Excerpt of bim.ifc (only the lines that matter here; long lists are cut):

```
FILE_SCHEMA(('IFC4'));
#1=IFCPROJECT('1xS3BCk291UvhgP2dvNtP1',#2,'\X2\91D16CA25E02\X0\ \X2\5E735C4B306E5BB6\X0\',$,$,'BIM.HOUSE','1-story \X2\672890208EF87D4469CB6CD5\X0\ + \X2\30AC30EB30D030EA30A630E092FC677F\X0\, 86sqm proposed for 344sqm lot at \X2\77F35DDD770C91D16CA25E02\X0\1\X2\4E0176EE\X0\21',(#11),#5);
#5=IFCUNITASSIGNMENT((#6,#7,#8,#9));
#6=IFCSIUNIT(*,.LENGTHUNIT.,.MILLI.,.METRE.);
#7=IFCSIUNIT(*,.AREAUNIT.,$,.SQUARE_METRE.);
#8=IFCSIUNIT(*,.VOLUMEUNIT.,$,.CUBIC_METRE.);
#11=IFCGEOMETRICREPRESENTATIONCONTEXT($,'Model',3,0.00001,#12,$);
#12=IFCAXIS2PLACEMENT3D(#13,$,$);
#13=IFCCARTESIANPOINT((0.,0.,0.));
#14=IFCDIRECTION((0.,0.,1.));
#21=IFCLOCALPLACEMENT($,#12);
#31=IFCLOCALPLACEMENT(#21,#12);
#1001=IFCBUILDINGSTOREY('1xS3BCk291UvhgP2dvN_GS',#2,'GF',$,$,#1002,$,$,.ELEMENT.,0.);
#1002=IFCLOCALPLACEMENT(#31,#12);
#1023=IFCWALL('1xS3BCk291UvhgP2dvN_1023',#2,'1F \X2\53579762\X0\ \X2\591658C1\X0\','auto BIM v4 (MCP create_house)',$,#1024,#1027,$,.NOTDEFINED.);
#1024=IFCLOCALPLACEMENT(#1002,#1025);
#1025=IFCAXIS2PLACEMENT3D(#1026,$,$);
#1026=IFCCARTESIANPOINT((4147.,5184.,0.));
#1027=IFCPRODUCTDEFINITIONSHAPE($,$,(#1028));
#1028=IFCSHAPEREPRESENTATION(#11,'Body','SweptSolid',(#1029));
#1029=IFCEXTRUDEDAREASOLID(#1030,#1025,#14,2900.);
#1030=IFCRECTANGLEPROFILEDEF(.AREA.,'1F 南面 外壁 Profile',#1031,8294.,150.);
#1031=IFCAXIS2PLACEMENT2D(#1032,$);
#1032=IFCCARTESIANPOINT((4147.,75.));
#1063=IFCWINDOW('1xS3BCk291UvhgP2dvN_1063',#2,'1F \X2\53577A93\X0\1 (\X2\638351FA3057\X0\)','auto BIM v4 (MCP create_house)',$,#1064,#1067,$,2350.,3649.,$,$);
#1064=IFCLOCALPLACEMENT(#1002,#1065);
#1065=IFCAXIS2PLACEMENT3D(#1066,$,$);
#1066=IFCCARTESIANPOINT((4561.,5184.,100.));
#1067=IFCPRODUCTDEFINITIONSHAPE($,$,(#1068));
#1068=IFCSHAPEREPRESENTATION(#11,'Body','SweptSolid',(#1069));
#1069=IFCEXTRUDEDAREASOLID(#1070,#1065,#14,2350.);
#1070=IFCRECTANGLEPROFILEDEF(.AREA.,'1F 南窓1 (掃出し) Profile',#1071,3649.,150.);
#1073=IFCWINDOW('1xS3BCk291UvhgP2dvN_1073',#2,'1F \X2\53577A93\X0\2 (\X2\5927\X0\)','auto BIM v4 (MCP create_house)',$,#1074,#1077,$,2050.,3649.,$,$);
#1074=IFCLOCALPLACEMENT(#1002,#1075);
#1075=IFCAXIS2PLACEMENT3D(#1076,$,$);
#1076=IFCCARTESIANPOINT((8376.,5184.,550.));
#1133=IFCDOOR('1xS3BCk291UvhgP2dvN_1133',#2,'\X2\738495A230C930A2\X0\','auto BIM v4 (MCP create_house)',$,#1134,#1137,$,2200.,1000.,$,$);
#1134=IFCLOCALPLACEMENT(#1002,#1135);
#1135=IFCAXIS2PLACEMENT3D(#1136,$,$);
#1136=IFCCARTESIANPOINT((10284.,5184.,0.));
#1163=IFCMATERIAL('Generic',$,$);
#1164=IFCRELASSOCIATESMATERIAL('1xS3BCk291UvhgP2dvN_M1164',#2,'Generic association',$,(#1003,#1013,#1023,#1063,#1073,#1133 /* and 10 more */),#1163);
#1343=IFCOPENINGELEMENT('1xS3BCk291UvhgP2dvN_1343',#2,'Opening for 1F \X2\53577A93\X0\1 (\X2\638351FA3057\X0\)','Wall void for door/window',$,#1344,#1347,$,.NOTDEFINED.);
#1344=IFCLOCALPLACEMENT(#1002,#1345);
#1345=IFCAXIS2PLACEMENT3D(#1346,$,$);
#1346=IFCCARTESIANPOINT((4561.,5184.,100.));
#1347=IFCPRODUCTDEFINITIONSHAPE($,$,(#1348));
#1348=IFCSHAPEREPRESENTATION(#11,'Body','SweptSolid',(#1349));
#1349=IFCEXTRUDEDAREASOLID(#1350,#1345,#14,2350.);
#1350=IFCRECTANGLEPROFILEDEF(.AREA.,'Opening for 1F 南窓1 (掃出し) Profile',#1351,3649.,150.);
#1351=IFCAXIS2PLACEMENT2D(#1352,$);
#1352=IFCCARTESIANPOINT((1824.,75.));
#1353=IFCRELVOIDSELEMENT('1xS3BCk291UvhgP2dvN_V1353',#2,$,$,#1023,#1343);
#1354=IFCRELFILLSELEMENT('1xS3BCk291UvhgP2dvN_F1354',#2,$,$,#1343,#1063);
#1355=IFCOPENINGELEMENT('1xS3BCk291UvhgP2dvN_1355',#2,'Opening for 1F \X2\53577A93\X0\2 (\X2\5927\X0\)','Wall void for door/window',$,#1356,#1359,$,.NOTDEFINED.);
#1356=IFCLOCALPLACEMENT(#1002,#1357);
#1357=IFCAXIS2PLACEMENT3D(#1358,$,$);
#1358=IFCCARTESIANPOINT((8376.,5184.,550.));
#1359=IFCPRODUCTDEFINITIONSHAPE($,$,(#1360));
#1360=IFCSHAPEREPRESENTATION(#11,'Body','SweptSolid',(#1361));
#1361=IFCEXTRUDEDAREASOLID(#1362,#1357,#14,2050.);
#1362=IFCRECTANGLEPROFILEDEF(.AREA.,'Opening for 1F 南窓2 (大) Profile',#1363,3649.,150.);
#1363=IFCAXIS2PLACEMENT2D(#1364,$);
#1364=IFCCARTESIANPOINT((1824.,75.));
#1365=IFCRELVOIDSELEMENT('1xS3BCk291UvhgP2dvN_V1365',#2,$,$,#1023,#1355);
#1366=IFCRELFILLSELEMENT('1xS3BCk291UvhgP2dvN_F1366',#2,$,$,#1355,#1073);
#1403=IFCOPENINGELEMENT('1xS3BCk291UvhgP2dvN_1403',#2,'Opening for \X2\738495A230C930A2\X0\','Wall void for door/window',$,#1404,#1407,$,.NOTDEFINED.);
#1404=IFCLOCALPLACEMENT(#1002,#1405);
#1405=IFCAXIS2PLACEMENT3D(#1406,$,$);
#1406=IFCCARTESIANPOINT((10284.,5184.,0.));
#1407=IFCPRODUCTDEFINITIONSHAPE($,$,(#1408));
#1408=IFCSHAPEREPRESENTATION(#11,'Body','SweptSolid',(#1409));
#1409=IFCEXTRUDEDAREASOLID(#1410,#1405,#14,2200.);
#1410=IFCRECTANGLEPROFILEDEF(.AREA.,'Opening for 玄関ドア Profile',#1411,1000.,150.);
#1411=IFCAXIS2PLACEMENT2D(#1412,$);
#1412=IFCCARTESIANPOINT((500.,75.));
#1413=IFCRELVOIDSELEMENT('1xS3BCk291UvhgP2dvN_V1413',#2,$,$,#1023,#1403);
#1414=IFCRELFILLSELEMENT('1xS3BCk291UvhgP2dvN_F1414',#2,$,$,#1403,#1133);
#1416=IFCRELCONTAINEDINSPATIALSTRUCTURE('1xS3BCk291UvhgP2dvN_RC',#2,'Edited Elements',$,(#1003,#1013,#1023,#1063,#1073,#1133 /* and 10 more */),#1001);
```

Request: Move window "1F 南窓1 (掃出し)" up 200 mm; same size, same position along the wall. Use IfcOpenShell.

```python
import numpy as np
import ifcopenshell
import ifcopenshell.api.geometry
import ifcopenshell.util.placement
import ifcopenshell.util.unit

model = ifcopenshell.open("bim.ifc")
unit_scale = ifcopenshell.util.unit.calculate_unit_scale(model)

window = model.by_id(1063)
opening = window.FillsVoids[0].RelatingOpeningElement
dz = 200.0

shift = np.array([0.0, 0.0, dz])
# The window is not placed relative to its opening, so move both.
for product in (opening, window):
    matrix = ifcopenshell.util.placement.get_local_placement(product.ObjectPlacement)
    matrix[:3, 3] += shift
    ifcopenshell.api.geometry.edit_object_placement(model, product=product, matrix=matrix, is_si=False)

print(f"moved by {dz * unit_scale:+.3f} m")

model.write("bim_updated.ifc")
```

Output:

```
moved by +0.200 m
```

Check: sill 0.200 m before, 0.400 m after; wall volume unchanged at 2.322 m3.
